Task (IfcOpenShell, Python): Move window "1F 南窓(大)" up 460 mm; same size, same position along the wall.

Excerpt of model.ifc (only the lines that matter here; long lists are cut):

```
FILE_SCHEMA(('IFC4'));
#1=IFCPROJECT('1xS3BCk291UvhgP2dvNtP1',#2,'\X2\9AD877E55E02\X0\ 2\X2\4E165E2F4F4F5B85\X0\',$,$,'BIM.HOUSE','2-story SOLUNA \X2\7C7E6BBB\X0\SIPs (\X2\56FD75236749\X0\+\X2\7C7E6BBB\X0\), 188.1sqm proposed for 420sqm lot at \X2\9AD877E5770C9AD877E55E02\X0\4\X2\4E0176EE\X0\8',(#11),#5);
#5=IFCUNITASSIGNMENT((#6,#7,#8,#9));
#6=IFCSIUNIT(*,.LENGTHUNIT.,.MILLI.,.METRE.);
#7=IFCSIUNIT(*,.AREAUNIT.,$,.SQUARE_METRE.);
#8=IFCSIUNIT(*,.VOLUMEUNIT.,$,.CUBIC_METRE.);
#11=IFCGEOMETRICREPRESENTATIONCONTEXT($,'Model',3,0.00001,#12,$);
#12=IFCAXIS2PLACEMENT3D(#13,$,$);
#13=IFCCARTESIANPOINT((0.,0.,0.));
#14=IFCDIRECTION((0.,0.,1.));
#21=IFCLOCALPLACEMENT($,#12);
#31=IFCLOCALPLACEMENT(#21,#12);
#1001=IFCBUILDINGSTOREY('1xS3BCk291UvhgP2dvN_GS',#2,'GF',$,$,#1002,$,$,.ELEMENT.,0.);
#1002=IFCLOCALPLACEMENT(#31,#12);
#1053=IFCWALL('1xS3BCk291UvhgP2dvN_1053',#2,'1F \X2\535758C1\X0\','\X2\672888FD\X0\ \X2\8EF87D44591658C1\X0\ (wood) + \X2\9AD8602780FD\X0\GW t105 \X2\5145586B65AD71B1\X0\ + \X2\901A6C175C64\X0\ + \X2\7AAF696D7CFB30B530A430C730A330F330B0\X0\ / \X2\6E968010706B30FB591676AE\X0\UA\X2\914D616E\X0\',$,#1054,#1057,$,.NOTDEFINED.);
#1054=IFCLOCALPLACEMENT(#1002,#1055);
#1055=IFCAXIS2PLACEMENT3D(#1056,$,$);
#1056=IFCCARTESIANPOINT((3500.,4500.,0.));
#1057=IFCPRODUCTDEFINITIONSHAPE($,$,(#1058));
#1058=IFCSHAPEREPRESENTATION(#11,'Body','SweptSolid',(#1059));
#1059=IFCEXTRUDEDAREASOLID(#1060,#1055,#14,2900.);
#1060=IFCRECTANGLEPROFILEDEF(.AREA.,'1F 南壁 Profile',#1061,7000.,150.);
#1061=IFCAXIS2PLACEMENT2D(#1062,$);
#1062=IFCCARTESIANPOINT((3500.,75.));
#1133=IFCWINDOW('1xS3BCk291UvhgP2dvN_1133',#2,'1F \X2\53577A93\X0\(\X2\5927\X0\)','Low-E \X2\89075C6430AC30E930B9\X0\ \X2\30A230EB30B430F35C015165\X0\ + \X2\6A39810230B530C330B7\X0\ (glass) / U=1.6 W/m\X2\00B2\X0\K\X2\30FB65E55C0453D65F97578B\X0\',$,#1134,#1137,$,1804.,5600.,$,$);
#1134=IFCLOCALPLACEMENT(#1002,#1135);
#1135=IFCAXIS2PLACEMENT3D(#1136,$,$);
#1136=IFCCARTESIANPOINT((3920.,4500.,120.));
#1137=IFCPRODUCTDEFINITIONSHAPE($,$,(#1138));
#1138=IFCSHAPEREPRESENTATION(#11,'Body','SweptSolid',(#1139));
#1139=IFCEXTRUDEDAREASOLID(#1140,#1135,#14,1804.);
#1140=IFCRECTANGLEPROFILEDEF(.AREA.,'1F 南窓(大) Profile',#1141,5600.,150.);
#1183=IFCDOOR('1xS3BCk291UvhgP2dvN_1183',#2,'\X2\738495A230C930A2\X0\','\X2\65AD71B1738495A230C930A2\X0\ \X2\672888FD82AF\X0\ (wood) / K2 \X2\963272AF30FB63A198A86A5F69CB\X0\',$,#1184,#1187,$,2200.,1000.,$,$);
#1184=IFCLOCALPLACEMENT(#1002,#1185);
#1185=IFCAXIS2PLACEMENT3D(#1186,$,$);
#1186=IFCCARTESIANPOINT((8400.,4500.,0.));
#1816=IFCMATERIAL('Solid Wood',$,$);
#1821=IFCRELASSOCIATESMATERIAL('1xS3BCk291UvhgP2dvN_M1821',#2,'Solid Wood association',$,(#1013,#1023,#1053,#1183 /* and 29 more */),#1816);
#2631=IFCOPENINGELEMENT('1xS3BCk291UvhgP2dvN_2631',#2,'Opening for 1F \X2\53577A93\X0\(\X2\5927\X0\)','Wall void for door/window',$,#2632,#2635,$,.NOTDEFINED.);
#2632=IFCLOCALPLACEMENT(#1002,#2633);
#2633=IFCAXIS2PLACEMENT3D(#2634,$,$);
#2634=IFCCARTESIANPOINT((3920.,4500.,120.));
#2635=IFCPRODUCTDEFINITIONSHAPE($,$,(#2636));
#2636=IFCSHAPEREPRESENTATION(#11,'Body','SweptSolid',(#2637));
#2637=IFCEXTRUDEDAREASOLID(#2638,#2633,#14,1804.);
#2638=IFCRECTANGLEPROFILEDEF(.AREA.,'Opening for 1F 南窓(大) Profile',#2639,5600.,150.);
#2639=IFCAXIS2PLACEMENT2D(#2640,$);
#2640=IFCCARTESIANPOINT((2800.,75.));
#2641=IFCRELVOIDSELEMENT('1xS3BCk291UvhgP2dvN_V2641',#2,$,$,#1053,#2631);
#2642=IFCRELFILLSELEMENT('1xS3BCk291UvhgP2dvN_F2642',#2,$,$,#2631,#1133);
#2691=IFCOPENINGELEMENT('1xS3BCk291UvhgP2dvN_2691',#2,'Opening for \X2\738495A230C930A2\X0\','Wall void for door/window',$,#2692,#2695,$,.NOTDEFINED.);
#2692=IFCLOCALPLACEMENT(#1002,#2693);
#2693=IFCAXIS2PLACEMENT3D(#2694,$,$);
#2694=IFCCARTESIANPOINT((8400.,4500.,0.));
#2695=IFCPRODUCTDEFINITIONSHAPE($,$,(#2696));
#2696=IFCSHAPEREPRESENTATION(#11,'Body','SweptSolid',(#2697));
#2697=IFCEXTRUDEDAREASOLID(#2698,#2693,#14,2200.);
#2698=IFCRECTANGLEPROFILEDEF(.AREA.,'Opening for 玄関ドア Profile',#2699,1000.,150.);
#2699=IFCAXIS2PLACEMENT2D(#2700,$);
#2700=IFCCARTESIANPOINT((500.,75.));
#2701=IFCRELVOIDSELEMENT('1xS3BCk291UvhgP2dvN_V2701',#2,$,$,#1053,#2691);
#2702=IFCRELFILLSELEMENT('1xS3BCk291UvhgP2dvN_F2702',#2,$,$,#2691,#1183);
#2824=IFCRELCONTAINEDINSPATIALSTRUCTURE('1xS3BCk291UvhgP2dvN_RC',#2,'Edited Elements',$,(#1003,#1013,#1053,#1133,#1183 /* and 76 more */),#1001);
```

```python
import numpy as np
import ifcopenshell
import ifcopenshell.api.geometry
import ifcopenshell.util.placement
import ifcopenshell.util.unit

model = ifcopenshell.open("model.ifc")
unit_scale = ifcopenshell.util.unit.calculate_unit_scale(model)

window = model.by_guid("1xS3BCk291UvhgP2dvN_1133")
opening = window.FillsVoids[0].RelatingOpeningElement
dz = 0.46 / unit_scale

shift = np.array([0.0, 0.0, dz])
# The window is not placed relative to its opening, so move both.
for product in (opening, window):
    matrix = ifcopenshell.util.placement.get_local_placement(product.ObjectPlacement)
    matrix[:3, 3] += shift
    ifcopenshell.api.geometry.edit_object_placement(model, product=product, matrix=matrix, is_si=False)

print(f"moved by {dz * unit_scale:+.3f} m")

model.write("model_edited.ifc")
```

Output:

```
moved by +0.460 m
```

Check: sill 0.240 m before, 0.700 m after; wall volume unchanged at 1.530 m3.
